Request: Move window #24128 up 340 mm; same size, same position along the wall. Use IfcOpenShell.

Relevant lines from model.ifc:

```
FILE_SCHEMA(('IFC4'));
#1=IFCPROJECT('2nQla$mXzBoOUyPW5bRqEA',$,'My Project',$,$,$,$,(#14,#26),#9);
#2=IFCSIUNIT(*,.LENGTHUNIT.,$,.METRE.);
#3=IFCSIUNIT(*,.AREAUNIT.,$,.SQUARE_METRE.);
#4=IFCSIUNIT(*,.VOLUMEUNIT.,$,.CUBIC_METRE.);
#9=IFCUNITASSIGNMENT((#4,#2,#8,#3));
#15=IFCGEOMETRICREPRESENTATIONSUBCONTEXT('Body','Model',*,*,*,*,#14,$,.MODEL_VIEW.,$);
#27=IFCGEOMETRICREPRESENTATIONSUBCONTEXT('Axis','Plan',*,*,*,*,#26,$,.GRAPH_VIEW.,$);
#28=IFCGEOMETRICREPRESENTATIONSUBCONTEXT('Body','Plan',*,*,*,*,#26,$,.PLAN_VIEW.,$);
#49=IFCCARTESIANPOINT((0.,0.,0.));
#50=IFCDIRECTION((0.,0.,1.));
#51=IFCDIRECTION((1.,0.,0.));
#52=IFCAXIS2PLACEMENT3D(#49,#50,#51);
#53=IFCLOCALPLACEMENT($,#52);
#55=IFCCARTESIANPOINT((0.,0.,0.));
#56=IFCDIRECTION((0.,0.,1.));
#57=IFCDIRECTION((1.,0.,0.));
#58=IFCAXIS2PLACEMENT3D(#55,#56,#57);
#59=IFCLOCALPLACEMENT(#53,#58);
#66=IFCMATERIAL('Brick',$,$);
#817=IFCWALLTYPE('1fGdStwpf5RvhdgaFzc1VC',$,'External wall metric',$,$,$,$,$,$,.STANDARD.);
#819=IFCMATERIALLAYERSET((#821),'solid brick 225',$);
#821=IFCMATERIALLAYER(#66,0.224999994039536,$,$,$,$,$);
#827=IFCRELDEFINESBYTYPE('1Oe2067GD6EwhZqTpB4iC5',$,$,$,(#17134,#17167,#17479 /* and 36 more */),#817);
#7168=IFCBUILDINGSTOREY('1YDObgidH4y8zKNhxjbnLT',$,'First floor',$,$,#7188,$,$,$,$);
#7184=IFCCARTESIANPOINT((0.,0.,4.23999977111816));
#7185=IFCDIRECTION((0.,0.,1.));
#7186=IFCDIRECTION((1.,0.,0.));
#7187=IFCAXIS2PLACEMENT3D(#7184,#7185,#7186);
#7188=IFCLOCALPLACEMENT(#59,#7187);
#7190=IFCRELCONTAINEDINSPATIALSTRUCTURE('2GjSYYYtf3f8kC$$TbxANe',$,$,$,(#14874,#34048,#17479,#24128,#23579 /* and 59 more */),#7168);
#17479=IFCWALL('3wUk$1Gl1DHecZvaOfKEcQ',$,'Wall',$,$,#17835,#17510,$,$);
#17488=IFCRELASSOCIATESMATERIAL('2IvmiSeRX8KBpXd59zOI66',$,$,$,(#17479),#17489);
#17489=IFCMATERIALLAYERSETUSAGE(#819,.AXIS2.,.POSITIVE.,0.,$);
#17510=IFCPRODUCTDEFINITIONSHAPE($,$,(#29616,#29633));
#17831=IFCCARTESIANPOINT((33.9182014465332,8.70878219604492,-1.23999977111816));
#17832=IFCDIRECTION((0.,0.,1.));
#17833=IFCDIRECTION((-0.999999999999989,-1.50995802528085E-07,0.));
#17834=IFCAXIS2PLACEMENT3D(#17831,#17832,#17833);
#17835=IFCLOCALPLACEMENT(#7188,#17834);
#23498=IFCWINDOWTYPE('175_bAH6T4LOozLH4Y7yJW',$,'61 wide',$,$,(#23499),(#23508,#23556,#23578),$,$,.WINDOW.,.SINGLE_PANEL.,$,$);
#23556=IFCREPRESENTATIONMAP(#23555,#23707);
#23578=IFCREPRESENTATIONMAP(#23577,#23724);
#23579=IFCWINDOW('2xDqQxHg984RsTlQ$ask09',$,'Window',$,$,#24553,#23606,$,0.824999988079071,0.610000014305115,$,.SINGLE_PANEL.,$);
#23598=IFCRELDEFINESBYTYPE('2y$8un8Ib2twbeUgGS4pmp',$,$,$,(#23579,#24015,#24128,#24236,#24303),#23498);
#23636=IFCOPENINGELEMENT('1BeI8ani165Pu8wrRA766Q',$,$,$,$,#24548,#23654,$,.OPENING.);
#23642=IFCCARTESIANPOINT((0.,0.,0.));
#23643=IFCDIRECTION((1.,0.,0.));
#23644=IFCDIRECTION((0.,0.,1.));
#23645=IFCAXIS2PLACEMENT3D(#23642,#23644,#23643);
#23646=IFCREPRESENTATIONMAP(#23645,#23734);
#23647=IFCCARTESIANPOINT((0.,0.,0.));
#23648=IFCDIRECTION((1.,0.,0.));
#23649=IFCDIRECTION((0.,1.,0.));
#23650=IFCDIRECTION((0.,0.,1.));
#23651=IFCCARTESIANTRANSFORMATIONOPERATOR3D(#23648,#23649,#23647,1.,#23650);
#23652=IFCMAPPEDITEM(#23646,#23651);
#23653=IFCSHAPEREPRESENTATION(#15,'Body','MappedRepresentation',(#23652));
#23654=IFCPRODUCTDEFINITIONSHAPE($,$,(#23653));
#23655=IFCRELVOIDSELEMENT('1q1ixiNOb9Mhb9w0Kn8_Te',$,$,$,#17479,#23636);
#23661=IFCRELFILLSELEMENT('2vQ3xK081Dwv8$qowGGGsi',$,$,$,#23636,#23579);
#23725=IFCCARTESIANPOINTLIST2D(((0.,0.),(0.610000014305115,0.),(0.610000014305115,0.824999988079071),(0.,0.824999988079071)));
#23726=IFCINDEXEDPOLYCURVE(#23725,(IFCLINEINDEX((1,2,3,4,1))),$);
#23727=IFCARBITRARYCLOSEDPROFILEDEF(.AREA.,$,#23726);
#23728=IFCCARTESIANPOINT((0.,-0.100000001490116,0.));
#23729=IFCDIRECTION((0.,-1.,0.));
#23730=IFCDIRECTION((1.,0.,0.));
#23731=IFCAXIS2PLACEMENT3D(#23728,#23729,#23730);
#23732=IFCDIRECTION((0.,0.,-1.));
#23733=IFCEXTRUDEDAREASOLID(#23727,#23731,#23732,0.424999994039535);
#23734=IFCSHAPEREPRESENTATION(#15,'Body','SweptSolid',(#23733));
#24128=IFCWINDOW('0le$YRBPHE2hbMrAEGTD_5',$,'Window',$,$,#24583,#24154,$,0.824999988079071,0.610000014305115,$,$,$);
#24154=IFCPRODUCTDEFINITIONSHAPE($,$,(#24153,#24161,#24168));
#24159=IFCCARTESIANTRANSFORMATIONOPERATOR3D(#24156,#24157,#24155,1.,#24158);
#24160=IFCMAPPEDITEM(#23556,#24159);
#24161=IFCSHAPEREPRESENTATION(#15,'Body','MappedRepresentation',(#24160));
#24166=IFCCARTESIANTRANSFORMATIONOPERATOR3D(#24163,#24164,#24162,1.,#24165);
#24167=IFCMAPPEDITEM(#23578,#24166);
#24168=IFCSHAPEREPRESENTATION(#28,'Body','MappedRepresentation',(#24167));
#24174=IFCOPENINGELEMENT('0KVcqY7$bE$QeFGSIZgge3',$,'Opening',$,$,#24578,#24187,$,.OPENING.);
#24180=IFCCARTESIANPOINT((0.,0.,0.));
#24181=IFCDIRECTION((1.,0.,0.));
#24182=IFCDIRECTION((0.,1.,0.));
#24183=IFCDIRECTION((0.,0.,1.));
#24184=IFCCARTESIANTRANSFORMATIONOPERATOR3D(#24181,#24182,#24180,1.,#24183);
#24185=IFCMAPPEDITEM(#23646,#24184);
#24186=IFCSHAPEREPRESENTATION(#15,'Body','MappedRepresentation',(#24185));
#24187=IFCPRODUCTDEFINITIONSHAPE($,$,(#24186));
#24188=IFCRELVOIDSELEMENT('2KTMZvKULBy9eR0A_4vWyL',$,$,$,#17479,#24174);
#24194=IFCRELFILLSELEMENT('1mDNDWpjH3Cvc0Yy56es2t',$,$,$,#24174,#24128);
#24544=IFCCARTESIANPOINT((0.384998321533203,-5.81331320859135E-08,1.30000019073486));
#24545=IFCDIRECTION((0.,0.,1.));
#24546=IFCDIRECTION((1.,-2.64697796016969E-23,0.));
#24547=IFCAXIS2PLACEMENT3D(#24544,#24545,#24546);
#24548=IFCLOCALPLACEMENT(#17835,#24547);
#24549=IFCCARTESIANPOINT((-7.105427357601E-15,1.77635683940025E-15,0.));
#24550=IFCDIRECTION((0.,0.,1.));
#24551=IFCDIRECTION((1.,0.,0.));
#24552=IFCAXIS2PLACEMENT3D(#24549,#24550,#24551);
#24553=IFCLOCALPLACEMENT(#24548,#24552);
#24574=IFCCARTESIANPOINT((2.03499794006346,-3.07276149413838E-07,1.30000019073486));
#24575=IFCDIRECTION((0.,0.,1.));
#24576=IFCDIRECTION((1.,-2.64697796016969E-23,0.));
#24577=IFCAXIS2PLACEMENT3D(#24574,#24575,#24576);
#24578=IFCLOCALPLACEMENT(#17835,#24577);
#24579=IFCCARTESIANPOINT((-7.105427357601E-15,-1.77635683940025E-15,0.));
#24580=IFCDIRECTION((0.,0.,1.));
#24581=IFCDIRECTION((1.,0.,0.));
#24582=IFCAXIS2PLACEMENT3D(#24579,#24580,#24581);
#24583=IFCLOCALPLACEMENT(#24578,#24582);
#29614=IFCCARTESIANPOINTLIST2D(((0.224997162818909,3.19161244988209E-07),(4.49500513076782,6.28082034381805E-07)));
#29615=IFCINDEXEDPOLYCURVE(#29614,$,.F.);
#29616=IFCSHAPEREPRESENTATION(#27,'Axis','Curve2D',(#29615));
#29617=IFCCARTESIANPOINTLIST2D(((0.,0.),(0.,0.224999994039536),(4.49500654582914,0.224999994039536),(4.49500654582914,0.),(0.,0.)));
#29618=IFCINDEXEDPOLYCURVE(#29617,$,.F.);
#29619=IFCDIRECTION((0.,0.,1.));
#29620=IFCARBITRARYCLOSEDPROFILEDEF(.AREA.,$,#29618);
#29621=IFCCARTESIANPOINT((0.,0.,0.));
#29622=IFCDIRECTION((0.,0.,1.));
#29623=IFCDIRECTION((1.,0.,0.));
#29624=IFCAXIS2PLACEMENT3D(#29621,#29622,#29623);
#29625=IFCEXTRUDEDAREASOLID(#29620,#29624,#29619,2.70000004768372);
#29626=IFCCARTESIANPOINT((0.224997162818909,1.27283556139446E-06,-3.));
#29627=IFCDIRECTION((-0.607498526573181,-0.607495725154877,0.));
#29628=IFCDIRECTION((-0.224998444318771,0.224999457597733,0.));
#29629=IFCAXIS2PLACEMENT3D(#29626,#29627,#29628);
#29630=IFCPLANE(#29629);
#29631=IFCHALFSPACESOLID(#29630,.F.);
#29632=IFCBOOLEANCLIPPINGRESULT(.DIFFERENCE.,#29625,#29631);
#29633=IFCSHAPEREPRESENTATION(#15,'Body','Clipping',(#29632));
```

```python
import numpy as np
import ifcopenshell
import ifcopenshell.api.geometry
import ifcopenshell.util.placement
import ifcopenshell.util.unit

model = ifcopenshell.open("model.ifc")
unit_scale = ifcopenshell.util.unit.calculate_unit_scale(model)

window = model.by_guid("0le$YRBPHE2hbMrAEGTD_5")
opening = window.FillsVoids[0].RelatingOpeningElement
dz = 0.34 / unit_scale

shift = np.array([0.0, 0.0, dz])
# The window is placed relative to its opening, so it follows when the opening moves.
matrix = ifcopenshell.util.placement.get_local_placement(opening.ObjectPlacement)
matrix[:3, 3] += shift
ifcopenshell.api.geometry.edit_object_placement(
    model, product=opening, matrix=matrix, is_si=False, should_transform_children=True
)

print(f"moved by {dz * unit_scale:+.3f} m")

model.write("model-out.ifc")
```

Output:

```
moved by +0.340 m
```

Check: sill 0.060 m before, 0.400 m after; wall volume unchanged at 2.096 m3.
